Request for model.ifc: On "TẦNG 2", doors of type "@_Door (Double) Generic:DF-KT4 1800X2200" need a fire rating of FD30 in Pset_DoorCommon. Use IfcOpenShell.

First a look at what the model holds.

```python
import ifcopenshell
import ifcopenshell.util.element

model = ifcopenshell.open("model.ifc")
print(model.schema)
storey = next(s for s in model.by_type("IfcBuildingStorey") if s.Name == "TẦNG 2")
doors = [e for e in ifcopenshell.util.element.get_decomposition(storey) if e.is_a("IfcDoor")]
seen = {}
for e in doors:
    element_type = ifcopenshell.util.element.get_type(e)
    key = (element_type.Name if element_type != e and element_type else None, ifcopenshell.util.element.get_pset(e, "Pset_DoorCommon", "FireRating"))
    seen[key] = seen.get(key, 0) + 1
for (name, value), count in sorted(seen.items(), key=str):
    print(count, "x", name, "|", value)
```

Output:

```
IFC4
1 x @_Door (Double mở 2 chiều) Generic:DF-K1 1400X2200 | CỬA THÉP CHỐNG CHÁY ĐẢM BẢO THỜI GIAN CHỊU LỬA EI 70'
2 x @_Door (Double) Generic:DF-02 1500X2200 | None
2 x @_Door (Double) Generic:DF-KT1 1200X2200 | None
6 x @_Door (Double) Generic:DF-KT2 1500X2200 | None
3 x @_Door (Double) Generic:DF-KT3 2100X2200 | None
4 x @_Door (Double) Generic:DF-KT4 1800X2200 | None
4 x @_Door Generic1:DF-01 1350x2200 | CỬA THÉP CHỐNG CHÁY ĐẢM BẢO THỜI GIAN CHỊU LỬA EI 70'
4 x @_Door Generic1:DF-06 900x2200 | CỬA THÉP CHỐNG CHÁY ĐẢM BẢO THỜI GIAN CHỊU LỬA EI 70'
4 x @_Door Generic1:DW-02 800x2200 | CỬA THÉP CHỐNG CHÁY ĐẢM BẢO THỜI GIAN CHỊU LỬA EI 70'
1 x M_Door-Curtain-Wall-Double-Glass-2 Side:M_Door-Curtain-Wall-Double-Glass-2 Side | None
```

```python
import ifcopenshell
import ifcopenshell.api.pset
import ifcopenshell.util.element

model = ifcopenshell.open("model.ifc")

storey = next(s for s in model.by_type("IfcBuildingStorey") if s.Name == "TẦNG 2")
doors = [e for e in ifcopenshell.util.element.get_decomposition(storey) if e.is_a("IfcDoor")]

count = 0
for e in doors:
    element_type = ifcopenshell.util.element.get_type(e)
    if element_type in (None, e) or element_type.Name != "@_Door (Double) Generic:DF-KT4 1800X2200":
        continue
    # add_pset returns the element's existing set when there is one.
    pset = ifcopenshell.api.pset.add_pset(model, product=e, name="Pset_DoorCommon")
    ifcopenshell.api.pset.edit_pset(model, pset=pset, properties={"FireRating": "FD30"})
    count += 1

print(count, "doors updated")

model.write("model_rev.ifc")
```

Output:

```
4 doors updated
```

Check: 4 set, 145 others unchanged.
